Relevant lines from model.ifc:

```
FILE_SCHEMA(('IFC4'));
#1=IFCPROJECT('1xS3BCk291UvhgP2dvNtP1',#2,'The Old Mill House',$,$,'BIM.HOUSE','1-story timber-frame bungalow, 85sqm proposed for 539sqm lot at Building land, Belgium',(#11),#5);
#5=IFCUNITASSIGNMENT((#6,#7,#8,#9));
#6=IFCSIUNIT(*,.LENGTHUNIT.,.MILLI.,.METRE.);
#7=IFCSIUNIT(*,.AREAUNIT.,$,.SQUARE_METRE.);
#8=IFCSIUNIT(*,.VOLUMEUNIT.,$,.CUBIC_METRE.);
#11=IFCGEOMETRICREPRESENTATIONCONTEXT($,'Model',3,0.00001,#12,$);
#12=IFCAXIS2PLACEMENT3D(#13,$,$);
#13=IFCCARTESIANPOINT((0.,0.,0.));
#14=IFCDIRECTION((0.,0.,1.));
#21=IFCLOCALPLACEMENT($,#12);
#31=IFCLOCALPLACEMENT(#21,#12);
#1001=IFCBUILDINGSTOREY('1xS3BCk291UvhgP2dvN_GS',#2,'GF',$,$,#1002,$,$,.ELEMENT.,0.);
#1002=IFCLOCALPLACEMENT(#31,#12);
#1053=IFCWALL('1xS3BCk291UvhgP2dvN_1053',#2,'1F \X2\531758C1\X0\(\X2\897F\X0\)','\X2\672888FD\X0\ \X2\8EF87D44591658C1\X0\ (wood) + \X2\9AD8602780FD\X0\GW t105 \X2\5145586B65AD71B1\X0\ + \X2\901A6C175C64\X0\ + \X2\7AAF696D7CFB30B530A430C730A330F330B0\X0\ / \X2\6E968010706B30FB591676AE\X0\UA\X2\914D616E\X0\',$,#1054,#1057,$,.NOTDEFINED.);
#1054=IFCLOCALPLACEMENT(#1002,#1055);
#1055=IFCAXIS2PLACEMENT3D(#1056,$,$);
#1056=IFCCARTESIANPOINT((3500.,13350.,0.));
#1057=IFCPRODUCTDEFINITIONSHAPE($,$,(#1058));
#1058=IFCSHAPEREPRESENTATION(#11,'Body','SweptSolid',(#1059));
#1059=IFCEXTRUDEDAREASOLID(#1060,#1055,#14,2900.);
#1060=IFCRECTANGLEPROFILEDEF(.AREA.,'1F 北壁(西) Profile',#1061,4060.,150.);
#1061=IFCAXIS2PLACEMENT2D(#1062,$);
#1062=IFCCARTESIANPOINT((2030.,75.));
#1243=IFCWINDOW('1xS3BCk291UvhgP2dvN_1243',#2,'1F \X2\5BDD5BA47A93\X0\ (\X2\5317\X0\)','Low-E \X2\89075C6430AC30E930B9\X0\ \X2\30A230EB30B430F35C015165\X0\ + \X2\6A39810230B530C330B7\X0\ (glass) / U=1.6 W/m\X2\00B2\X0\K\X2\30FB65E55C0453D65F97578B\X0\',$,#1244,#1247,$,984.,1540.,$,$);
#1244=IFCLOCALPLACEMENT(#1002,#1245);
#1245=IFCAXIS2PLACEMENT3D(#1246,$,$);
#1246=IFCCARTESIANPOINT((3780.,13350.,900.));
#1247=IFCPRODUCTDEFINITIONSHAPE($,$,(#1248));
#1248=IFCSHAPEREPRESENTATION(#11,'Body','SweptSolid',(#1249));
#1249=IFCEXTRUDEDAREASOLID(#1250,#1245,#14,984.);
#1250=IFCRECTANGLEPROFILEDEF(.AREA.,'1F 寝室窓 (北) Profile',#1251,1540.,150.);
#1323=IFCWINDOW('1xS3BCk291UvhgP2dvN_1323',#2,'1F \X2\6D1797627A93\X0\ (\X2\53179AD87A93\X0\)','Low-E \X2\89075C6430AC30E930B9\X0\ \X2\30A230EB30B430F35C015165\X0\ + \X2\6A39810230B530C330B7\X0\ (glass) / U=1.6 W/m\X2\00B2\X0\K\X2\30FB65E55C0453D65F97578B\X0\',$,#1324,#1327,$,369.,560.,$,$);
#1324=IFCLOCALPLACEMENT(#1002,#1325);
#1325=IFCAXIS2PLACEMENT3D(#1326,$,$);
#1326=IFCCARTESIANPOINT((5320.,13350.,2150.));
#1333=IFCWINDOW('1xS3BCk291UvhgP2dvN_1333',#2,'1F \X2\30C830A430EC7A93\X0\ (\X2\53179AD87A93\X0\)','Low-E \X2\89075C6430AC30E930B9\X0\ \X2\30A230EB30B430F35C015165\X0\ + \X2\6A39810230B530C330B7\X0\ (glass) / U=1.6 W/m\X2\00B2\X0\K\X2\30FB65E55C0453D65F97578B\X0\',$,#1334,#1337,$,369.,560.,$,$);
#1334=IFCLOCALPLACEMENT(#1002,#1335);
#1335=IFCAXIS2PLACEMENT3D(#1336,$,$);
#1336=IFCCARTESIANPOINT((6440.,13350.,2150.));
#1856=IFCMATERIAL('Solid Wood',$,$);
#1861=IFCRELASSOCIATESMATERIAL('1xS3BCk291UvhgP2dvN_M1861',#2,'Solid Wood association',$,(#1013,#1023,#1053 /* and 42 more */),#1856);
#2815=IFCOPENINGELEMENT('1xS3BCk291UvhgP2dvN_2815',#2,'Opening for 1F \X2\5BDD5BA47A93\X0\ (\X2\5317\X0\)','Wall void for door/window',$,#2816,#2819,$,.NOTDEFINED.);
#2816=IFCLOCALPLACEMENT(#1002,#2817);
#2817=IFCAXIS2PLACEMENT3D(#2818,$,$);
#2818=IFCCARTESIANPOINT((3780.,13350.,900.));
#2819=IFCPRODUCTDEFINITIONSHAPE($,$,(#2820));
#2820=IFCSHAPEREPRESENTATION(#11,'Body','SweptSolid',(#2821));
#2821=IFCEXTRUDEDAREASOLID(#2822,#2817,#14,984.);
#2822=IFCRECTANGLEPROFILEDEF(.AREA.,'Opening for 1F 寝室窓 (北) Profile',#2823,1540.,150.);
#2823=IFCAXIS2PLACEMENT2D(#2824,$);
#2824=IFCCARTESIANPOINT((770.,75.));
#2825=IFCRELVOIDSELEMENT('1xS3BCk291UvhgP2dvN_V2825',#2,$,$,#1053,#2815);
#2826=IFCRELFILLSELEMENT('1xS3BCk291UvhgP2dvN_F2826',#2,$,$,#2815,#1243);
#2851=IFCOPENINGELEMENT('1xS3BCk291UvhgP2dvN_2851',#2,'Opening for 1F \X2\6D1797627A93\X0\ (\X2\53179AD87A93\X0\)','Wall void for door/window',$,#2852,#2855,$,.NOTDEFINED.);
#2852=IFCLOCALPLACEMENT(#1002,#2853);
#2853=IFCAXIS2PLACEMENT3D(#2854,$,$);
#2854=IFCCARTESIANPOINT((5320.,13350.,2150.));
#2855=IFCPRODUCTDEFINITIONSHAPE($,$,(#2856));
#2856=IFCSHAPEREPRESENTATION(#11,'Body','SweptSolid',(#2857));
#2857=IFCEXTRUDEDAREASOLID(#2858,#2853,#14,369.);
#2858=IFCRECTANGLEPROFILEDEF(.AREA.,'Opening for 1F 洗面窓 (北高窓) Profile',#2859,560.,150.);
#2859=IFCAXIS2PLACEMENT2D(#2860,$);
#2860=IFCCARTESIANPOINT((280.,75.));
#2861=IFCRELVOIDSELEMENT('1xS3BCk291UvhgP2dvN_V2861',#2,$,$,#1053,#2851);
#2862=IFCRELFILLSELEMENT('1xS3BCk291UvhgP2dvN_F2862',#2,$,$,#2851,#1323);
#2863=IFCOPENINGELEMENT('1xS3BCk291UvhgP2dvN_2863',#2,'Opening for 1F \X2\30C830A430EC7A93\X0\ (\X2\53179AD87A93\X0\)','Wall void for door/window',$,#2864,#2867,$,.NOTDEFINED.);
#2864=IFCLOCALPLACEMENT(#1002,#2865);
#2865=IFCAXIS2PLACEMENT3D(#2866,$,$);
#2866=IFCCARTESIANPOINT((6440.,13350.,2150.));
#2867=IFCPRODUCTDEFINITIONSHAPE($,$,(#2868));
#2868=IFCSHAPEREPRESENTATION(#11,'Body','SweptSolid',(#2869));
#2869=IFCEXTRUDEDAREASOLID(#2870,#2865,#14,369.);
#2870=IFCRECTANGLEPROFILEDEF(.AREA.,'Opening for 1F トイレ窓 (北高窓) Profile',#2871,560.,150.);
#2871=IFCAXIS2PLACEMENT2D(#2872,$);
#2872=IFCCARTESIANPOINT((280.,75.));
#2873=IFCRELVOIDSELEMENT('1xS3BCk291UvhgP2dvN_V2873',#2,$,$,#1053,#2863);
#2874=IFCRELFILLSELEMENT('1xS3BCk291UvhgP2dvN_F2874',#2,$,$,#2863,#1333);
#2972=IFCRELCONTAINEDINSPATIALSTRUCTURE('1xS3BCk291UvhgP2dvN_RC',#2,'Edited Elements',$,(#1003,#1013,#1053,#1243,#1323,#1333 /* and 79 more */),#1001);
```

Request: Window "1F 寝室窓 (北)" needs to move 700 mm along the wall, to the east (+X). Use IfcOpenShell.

```python
import ifcopenshell
import ifcopenshell.api.geometry
import ifcopenshell.util.placement
import ifcopenshell.util.unit

model = ifcopenshell.open("model.ifc")
unit_scale = ifcopenshell.util.unit.calculate_unit_scale(model)

window = model.by_guid("1xS3BCk291UvhgP2dvN_1243")
opening = window.FillsVoids[0].RelatingOpeningElement
wall = opening.VoidsElements[0].RelatingBuildingElement

wall_matrix = ifcopenshell.util.placement.get_local_placement(wall.ObjectPlacement)
shift = wall_matrix[:3, 0] * 0.7 / unit_scale
before = ifcopenshell.util.placement.get_local_placement(window.ObjectPlacement)[:3, 3].copy()

# The window is not placed relative to its opening, so move both.
for product in (opening, window):
    matrix = ifcopenshell.util.placement.get_local_placement(product.ObjectPlacement)
    matrix[:3, 3] += shift
    ifcopenshell.api.geometry.edit_object_placement(model, product=product, matrix=matrix, is_si=False)

after = ifcopenshell.util.placement.get_local_placement(window.ObjectPlacement)[:3, 3]
print("window moved by", (after - before).round(3) + 0.0)

model.write("model_updated.ifc")
```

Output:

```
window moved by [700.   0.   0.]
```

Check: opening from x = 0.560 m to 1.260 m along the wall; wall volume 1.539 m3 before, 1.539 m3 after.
